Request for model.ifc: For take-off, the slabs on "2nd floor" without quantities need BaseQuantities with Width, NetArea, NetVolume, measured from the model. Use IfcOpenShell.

First a look at what the model holds.

```python
import ifcopenshell
import ifcopenshell.util.element
import ifcopenshell.util.unit

model = ifcopenshell.open("model.ifc")
print(model.schema)
for unit_type in ("LENGTHUNIT", "AREAUNIT", "VOLUMEUNIT"):
    print(unit_type, ifcopenshell.util.unit.calculate_unit_scale(model, unit_type))
storey = next(s for s in model.by_type("IfcBuildingStorey") if s.Name == "2nd floor")
slabs = [e for e in ifcopenshell.util.element.get_decomposition(storey) if e.is_a("IfcSlab")]
for e in sorted(slabs, key=lambda e: e.id()):
    print(e.id(), e.is_a(), e.Name, list(ifcopenshell.util.element.get_psets(e, qtos_only=True)), sep=" | ")
```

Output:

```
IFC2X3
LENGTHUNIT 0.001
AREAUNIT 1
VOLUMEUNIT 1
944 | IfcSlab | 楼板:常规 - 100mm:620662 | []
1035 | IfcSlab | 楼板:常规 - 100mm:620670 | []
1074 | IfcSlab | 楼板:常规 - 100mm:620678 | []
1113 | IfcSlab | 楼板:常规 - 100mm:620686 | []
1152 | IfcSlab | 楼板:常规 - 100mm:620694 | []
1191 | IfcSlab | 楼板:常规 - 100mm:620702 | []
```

```python
import ifcopenshell
import ifcopenshell.api.pset
import ifcopenshell.geom
import ifcopenshell.util.element
import ifcopenshell.util.shape
import ifcopenshell.util.unit

model = ifcopenshell.open("model.ifc")
unit_scale = ifcopenshell.util.unit.calculate_unit_scale(model)
area_scale = ifcopenshell.util.unit.calculate_unit_scale(model, "AREAUNIT")
volume_scale = ifcopenshell.util.unit.calculate_unit_scale(model, "VOLUMEUNIT")
settings = ifcopenshell.geom.settings()

storey = next(s for s in model.by_type("IfcBuildingStorey") if s.Name == "2nd floor")
slabs = [e for e in ifcopenshell.util.element.get_decomposition(storey) if e.is_a("IfcSlab")]

for e in sorted(slabs, key=lambda e: e.id()):
    if ifcopenshell.util.element.get_psets(e, qtos_only=True, should_inherit=False):
        continue
    # Geometry comes back in metres, in the element's own axes.
    shape = ifcopenshell.geom.create_shape(settings, e)
    values = {
        "Width": ifcopenshell.util.shape.get_z(shape.geometry) / unit_scale,
        "NetArea": ifcopenshell.util.shape.get_footprint_area(shape.geometry) / area_scale,
        "NetVolume": ifcopenshell.util.shape.get_volume(shape.geometry) / volume_scale,
    }
    qto = ifcopenshell.api.pset.add_qto(model, product=e, name="BaseQuantities")
    ifcopenshell.api.pset.edit_qto(model, qto=qto, properties=values)
    print(e.id(), {k: round(v, 3) for k, v in values.items()})

model.write("model_v2.ifc")
```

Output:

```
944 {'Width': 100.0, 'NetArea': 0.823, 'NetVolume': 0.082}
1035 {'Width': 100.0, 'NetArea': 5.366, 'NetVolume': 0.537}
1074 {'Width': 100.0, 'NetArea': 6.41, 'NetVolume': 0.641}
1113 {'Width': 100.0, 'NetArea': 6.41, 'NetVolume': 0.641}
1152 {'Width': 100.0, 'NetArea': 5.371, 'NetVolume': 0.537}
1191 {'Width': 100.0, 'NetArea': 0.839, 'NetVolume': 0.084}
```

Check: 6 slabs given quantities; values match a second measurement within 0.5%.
